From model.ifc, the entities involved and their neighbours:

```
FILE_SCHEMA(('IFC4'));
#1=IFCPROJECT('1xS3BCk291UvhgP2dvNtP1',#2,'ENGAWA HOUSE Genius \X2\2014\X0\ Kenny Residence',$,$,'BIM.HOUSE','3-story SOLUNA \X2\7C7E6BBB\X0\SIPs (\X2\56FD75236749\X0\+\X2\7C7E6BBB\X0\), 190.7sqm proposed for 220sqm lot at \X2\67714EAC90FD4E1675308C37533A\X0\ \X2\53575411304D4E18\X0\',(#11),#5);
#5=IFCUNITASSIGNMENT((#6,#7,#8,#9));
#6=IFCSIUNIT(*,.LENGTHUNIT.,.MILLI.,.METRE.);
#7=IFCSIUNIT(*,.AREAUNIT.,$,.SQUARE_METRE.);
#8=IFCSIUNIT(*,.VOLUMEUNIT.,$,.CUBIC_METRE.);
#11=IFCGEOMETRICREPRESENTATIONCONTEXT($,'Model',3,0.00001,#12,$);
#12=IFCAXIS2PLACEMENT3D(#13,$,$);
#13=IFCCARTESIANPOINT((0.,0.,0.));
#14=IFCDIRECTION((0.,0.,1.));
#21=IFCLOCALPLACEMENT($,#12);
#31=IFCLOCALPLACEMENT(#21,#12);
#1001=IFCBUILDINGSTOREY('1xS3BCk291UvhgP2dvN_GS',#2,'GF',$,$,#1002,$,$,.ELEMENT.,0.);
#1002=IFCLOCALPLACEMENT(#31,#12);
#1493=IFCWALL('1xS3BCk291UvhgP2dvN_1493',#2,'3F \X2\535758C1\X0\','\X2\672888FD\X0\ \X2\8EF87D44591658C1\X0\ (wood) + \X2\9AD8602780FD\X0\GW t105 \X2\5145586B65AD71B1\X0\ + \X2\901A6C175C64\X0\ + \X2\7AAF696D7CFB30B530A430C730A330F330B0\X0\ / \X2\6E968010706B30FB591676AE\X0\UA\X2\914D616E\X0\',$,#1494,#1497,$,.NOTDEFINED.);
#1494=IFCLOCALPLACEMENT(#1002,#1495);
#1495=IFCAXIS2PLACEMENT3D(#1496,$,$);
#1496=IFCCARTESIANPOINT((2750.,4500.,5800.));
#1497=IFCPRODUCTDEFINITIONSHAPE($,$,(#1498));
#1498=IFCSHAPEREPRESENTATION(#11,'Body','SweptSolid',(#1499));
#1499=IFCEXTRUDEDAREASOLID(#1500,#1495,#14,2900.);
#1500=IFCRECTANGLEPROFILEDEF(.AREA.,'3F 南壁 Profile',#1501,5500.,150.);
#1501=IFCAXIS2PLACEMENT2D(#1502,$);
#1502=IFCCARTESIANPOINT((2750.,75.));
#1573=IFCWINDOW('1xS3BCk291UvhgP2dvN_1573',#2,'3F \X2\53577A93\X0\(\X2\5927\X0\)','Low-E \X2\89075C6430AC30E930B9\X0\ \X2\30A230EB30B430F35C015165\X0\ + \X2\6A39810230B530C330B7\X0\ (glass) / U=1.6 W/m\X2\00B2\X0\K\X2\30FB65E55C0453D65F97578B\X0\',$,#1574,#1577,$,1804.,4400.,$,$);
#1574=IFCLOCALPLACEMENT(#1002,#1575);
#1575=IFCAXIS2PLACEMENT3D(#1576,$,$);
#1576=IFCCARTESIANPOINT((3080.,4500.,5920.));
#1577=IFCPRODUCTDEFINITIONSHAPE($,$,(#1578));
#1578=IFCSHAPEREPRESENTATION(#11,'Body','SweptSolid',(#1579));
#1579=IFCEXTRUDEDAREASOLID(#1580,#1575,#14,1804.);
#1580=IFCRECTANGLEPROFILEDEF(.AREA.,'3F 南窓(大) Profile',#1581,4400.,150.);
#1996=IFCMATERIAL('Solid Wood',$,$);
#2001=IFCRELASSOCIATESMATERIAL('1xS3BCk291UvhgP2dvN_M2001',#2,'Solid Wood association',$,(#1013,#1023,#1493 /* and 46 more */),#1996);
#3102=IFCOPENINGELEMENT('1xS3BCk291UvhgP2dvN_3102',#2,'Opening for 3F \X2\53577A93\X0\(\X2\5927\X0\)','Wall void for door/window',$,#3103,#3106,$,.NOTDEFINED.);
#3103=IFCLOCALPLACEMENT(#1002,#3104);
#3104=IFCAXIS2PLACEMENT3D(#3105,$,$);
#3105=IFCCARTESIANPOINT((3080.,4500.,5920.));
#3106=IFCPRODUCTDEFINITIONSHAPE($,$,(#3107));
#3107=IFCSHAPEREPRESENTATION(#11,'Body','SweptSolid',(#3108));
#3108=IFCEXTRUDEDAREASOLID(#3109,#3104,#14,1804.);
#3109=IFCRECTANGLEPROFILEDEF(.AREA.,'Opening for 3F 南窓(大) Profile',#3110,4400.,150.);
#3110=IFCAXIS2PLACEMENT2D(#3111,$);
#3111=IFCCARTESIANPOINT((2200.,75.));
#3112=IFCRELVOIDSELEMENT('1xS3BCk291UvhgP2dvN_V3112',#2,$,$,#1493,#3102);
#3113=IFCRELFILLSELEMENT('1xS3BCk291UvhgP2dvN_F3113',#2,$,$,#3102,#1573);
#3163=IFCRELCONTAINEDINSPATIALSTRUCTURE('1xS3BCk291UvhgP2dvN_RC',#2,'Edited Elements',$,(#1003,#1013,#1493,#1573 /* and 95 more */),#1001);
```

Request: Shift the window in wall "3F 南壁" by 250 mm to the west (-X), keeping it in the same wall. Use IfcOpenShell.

```python
import ifcopenshell
import ifcopenshell.api.geometry
import ifcopenshell.util.placement

model = ifcopenshell.open("model.ifc")

window = model.by_guid("1xS3BCk291UvhgP2dvN_1573")
opening = window.FillsVoids[0].RelatingOpeningElement
wall = opening.VoidsElements[0].RelatingBuildingElement

wall_matrix = ifcopenshell.util.placement.get_local_placement(wall.ObjectPlacement)
shift = wall_matrix[:3, 0] * -250.0
before = ifcopenshell.util.placement.get_local_placement(window.ObjectPlacement)[:3, 3].copy()

# The window is not placed relative to its opening, so move both.
for product in (opening, window):
    matrix = ifcopenshell.util.placement.get_local_placement(product.ObjectPlacement)
    matrix[:3, 3] += shift
    ifcopenshell.api.geometry.edit_object_placement(model, product=product, matrix=matrix, is_si=False)

after = ifcopenshell.util.placement.get_local_placement(window.ObjectPlacement)[:3, 3]
print("window moved by", (after - before).round(3) + 0.0)

model.write("model_v2.ifc")
```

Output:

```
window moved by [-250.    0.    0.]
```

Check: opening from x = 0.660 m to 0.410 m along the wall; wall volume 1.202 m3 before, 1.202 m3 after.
